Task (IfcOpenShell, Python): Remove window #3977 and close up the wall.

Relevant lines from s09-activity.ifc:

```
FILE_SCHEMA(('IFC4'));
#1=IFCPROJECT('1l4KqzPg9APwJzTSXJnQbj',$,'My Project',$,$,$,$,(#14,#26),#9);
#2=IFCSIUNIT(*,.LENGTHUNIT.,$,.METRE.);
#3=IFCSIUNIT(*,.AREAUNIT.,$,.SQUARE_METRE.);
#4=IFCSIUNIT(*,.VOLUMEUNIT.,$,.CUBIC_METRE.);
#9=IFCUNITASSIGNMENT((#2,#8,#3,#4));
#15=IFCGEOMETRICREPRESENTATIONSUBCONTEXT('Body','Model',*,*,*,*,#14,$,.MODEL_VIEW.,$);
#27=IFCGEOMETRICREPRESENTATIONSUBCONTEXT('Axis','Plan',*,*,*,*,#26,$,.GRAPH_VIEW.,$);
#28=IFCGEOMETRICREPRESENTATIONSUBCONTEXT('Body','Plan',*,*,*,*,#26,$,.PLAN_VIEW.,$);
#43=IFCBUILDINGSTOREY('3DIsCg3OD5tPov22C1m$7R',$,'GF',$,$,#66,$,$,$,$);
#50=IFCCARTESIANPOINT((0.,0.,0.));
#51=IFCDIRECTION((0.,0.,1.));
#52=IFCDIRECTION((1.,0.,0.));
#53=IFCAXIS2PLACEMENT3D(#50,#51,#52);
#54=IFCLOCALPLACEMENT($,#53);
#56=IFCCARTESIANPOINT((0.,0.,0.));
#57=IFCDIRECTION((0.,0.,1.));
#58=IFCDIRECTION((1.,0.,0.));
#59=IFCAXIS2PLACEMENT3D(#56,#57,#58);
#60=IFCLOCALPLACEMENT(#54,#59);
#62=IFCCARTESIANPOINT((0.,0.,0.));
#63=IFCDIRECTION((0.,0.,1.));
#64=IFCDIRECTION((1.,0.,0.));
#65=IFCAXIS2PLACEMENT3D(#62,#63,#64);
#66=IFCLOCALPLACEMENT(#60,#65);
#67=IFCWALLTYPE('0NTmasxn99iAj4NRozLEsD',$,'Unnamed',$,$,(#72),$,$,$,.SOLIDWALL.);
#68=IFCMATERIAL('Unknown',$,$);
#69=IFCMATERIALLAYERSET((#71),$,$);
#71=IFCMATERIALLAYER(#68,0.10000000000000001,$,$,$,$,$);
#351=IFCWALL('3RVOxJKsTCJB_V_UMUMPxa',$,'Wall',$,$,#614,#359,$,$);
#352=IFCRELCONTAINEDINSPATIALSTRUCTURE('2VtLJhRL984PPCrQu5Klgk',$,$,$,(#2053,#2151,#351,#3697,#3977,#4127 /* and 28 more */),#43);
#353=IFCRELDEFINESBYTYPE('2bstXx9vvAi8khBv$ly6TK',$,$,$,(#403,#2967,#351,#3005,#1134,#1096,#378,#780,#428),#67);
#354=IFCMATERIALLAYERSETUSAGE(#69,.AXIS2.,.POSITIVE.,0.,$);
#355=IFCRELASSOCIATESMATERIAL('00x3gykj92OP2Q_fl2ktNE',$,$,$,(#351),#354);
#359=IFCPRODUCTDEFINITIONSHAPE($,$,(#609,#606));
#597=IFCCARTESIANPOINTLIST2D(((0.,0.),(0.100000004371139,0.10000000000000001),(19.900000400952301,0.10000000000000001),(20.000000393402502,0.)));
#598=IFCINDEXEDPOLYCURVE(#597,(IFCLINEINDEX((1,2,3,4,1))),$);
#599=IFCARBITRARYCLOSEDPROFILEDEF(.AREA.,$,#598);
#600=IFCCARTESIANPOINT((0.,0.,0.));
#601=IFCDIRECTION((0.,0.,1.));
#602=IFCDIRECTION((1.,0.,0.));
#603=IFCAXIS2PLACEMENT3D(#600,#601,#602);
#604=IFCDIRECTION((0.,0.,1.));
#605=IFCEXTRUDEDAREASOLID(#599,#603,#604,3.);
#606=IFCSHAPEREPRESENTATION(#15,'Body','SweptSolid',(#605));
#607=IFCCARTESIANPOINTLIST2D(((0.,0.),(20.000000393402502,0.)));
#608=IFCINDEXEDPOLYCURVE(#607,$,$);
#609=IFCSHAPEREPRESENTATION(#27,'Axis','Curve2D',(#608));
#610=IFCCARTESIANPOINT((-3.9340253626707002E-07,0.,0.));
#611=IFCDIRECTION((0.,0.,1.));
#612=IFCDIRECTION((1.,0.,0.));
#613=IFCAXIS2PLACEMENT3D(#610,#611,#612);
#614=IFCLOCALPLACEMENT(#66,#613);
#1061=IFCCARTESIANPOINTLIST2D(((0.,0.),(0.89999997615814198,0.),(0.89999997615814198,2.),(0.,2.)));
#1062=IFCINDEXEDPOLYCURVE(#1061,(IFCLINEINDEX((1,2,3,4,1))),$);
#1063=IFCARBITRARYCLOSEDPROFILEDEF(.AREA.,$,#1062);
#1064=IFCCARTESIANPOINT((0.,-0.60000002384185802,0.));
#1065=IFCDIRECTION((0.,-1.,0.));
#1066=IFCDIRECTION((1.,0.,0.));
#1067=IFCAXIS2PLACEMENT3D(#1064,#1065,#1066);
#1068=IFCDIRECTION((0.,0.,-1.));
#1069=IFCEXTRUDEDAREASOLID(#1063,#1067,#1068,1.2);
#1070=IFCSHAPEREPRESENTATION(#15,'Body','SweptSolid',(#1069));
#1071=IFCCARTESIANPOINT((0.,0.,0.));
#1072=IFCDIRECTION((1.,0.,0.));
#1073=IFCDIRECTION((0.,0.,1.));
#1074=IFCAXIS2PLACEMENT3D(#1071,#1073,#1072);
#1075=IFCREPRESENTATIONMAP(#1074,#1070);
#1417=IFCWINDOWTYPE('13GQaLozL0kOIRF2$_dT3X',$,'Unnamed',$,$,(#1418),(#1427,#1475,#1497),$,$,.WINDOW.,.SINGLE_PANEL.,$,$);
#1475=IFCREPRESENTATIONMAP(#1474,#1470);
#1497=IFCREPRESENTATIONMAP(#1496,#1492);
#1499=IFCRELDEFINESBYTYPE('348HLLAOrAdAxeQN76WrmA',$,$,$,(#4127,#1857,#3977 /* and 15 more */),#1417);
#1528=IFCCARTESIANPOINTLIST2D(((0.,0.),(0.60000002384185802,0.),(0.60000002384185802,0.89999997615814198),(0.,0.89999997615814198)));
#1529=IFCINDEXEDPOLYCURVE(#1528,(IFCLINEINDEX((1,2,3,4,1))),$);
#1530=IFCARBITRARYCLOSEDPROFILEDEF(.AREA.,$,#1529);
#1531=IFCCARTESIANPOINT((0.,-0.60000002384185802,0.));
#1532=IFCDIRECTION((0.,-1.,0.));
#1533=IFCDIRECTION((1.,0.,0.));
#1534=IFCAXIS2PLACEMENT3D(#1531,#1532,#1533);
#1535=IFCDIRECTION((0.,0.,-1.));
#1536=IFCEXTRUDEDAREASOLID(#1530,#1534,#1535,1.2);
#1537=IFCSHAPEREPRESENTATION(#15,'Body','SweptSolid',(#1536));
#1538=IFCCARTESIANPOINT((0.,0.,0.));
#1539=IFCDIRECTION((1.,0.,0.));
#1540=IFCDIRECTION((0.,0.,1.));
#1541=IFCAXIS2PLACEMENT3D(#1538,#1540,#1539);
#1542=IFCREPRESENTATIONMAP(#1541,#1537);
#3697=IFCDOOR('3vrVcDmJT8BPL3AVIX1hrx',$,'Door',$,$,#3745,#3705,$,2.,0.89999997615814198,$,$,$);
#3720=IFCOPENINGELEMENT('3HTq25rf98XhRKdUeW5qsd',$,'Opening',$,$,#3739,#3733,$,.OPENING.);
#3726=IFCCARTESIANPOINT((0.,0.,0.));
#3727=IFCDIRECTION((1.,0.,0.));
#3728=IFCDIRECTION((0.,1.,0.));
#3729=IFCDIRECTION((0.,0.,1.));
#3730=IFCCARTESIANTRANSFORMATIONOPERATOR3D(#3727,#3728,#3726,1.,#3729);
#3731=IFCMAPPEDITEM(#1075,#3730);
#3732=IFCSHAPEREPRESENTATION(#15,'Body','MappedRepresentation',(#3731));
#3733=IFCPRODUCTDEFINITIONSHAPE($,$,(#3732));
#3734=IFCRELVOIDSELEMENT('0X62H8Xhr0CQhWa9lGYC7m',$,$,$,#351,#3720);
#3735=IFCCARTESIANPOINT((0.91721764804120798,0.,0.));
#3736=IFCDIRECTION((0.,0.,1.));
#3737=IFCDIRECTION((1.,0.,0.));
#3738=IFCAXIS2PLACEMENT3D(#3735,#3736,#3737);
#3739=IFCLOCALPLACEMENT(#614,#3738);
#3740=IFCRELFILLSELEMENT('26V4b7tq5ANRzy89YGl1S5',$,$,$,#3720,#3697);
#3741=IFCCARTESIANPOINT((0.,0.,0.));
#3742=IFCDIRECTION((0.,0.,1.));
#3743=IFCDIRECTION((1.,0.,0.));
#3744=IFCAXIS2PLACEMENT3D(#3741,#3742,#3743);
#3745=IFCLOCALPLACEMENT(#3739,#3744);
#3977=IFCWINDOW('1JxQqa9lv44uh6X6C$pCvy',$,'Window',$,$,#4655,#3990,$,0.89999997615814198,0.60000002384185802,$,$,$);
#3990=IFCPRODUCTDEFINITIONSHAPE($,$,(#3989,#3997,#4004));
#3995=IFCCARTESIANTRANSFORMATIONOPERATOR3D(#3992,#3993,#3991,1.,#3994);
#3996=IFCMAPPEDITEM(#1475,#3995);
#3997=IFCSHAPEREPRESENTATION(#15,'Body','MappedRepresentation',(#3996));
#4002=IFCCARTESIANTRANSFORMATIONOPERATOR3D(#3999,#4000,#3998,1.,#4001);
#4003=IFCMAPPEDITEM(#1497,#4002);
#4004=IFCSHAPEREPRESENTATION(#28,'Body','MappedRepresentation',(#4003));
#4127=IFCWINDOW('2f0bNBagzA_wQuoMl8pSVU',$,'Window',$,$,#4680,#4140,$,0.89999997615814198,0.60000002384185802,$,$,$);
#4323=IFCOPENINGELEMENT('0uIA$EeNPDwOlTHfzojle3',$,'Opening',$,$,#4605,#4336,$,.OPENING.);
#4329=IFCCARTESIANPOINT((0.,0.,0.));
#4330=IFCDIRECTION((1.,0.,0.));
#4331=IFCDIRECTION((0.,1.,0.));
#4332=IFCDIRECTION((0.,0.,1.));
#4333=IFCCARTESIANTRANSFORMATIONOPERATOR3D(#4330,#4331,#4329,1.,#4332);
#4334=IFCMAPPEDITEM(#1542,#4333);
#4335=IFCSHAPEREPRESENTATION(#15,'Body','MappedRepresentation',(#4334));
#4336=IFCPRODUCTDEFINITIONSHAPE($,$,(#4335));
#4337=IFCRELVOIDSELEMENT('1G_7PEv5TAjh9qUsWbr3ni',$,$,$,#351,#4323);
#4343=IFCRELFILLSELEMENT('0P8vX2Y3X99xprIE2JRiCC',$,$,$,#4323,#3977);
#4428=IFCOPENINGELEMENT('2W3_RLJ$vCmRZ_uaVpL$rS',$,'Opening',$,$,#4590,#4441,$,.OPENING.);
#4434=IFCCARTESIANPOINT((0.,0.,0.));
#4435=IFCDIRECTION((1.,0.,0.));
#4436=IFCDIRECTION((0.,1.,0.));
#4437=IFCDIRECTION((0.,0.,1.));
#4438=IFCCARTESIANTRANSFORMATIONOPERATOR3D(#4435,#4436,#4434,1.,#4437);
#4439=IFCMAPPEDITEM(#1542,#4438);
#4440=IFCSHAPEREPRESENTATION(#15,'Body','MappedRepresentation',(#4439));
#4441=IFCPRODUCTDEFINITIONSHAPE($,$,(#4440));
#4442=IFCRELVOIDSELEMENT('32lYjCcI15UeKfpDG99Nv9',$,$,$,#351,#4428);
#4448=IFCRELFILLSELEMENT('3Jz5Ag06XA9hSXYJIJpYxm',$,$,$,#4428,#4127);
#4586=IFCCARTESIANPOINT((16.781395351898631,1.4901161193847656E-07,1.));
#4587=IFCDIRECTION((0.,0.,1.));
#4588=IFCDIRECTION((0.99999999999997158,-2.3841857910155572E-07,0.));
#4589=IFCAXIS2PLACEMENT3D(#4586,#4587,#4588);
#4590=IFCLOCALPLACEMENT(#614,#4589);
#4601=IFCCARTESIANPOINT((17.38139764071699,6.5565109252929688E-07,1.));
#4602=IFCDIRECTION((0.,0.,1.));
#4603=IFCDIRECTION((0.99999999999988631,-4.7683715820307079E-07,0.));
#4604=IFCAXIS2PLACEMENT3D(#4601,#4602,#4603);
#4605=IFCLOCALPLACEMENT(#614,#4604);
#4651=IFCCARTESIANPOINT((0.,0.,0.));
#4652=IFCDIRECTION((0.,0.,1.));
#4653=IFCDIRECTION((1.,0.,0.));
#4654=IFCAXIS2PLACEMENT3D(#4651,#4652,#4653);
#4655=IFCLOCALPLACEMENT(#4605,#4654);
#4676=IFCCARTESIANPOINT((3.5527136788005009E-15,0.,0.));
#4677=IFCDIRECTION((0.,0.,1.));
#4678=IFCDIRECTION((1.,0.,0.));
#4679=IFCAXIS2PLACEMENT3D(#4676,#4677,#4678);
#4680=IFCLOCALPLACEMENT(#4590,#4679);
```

```python
import ifcopenshell
import ifcopenshell.api.feature
import ifcopenshell.api.root
import ifcopenshell.geom
import ifcopenshell.util.shape

model = ifcopenshell.open("s09-activity.ifc")
settings = ifcopenshell.geom.settings()


def volume(element):
    """Net volume in cubic metres, openings subtracted."""
    shape = ifcopenshell.geom.create_shape(settings, element)
    return ifcopenshell.util.shape.get_volume(shape.geometry)


window = model.by_guid("1JxQqa9lv44uh6X6C$pCvy")
opening = window.FillsVoids[0].RelatingOpeningElement
wall = opening.VoidsElements[0].RelatingBuildingElement
before = volume(wall)

ifcopenshell.api.root.remove_product(model, product=window)
ifcopenshell.api.feature.remove_feature(model, feature=opening)

after = volume(wall)

print(f"wall volume {before:.3f} -> {after:.3f} m3")

model.write("s09-activity_v2.ifc")
```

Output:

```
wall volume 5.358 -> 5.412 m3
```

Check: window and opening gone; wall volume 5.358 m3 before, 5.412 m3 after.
